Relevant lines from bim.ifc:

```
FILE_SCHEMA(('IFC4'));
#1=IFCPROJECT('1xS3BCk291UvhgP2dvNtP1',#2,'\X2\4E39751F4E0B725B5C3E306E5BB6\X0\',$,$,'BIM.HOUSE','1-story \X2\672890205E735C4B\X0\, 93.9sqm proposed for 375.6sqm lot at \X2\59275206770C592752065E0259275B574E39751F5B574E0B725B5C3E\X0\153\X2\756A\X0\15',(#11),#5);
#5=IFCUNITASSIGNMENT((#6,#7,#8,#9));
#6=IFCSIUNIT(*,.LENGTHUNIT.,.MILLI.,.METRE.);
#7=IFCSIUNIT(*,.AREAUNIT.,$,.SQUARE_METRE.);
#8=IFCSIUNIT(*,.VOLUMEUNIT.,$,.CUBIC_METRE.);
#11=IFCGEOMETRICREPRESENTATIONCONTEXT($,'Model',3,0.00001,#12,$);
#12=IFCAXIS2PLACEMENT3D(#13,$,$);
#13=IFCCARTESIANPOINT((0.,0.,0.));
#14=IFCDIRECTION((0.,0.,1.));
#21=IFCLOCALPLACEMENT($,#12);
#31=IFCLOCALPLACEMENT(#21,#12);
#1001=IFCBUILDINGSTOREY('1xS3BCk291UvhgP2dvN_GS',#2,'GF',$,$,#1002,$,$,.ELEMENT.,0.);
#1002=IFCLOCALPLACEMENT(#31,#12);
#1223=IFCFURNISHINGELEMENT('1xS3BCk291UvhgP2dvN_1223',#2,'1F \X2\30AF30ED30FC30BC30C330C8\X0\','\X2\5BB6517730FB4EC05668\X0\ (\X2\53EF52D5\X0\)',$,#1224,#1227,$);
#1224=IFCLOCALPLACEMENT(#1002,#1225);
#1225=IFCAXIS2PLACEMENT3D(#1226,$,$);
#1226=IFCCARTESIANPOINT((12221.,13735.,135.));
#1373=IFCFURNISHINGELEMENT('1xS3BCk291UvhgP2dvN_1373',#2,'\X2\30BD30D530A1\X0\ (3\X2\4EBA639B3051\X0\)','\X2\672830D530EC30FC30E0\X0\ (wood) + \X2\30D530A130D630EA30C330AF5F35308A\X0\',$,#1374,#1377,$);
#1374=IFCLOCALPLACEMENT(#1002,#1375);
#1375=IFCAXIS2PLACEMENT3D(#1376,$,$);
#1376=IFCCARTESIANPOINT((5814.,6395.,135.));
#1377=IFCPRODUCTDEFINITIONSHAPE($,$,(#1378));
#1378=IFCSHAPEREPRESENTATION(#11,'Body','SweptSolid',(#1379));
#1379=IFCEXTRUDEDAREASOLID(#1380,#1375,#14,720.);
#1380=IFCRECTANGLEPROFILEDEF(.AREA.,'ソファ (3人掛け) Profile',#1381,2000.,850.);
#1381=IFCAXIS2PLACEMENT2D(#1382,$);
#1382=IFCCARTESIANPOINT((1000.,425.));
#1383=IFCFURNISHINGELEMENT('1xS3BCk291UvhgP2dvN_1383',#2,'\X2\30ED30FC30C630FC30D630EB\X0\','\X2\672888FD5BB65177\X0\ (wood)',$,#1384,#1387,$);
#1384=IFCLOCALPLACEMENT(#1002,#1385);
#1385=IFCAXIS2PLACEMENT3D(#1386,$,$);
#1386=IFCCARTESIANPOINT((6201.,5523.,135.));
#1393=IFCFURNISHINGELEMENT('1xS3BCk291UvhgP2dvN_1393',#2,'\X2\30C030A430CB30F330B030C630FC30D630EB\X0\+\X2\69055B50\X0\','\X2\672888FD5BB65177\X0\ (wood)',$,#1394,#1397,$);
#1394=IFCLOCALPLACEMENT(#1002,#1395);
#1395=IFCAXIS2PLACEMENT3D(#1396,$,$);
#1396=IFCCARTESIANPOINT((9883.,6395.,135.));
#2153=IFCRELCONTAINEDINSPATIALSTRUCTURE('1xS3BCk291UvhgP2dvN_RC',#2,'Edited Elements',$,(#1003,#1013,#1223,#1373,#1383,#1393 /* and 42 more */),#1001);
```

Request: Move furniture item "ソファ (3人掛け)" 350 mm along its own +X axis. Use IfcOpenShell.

```python
import ifcopenshell
import ifcopenshell.api.geometry
import ifcopenshell.util.placement
import ifcopenshell.util.unit

model = ifcopenshell.open("bim.ifc")
unit_scale = ifcopenshell.util.unit.calculate_unit_scale(model)

item = model.by_guid("1xS3BCk291UvhgP2dvN_1373")
matrix = ifcopenshell.util.placement.get_local_placement(item.ObjectPlacement)
matrix[:3, 3] += matrix[:3, 0] * 0.35 / unit_scale
ifcopenshell.api.geometry.edit_object_placement(model, product=item, matrix=matrix, is_si=False)

print(ifcopenshell.util.placement.get_local_placement(item.ObjectPlacement).round(3) + 0.0)

model.write("bim_edited.ifc")
```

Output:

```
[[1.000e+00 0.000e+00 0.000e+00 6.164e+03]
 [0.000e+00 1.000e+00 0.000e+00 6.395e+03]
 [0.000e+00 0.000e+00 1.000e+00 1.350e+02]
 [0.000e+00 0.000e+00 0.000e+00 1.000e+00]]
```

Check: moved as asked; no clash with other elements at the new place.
